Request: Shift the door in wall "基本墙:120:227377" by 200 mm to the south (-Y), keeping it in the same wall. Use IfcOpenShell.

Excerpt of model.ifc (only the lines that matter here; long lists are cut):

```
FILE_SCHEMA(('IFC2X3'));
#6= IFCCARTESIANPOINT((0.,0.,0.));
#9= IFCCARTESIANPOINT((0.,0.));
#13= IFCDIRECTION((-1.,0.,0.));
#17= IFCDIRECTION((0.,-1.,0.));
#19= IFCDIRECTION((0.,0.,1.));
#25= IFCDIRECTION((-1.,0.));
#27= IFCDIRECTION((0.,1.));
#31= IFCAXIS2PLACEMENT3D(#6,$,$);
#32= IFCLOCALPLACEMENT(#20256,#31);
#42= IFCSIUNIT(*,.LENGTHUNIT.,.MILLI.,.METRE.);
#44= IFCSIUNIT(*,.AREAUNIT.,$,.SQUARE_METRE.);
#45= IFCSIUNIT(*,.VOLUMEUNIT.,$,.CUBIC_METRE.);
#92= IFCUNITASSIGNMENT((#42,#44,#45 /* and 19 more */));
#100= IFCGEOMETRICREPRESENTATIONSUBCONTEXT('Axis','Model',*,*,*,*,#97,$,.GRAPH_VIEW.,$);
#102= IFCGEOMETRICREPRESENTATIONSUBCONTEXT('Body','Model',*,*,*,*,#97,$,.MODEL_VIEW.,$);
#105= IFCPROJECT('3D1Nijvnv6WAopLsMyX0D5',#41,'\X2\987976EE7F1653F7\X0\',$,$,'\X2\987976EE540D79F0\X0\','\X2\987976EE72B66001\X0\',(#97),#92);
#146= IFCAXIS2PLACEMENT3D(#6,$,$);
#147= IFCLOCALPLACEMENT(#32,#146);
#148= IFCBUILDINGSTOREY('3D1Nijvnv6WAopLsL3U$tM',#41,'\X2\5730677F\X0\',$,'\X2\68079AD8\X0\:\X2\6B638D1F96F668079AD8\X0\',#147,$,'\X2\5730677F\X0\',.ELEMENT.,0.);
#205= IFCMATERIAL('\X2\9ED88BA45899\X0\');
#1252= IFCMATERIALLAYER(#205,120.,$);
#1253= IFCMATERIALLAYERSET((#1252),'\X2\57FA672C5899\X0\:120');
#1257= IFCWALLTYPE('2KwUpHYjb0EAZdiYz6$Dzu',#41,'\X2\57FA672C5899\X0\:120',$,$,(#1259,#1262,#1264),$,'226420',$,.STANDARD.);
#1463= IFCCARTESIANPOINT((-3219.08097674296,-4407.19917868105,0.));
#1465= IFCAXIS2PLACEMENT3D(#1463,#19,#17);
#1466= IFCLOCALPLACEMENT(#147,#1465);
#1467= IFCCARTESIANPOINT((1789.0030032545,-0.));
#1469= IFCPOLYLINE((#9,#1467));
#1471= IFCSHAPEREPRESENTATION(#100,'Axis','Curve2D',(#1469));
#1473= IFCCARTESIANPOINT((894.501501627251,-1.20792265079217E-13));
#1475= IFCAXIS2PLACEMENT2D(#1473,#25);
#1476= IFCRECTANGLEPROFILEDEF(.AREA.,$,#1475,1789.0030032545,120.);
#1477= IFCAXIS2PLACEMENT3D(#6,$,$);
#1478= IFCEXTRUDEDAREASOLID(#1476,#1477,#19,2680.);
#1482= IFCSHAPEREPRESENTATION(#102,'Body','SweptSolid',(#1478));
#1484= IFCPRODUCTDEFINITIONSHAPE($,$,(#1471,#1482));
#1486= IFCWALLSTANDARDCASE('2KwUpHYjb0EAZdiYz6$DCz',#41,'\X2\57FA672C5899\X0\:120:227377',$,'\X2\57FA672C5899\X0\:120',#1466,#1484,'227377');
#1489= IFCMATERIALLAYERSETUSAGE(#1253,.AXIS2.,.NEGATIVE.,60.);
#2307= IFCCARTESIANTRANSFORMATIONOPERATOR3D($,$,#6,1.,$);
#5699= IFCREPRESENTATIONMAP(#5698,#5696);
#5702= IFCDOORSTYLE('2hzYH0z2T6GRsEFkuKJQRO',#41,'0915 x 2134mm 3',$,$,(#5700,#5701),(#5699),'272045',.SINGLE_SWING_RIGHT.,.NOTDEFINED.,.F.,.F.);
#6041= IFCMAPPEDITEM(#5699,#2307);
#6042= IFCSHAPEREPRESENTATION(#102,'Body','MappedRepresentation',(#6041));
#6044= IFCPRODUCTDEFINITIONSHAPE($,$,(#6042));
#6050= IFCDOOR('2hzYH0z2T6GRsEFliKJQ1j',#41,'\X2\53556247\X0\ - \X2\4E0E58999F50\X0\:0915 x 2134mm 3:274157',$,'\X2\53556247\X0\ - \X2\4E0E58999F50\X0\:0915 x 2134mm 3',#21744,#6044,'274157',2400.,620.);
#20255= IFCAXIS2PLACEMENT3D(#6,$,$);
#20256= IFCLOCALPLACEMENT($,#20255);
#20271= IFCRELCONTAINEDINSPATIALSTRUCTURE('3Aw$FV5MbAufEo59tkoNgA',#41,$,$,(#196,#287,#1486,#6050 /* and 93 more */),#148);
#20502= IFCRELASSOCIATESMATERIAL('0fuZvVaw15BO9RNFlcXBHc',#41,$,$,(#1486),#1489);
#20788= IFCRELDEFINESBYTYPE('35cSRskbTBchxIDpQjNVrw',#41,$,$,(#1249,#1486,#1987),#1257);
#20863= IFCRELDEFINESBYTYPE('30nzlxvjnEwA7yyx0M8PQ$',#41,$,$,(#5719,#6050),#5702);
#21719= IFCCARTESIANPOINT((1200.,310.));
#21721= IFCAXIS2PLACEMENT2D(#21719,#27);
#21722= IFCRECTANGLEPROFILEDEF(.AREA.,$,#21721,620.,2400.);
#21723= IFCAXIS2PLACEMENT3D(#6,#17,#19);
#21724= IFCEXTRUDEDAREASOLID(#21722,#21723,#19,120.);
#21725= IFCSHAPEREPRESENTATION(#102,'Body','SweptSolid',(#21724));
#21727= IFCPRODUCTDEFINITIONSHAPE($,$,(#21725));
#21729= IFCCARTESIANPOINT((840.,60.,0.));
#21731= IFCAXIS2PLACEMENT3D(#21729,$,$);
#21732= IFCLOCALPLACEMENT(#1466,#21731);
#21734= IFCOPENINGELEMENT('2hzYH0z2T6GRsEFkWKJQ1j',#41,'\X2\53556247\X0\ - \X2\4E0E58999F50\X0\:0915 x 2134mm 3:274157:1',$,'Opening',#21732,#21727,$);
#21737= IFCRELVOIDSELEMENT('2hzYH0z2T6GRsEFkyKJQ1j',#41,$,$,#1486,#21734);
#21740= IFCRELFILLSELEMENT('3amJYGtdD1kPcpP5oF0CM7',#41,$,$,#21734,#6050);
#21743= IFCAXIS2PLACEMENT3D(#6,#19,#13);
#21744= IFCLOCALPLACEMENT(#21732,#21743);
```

```python
import ifcopenshell
import ifcopenshell.api.geometry
import ifcopenshell.util.placement
import ifcopenshell.util.unit

model = ifcopenshell.open("model.ifc")
unit_scale = ifcopenshell.util.unit.calculate_unit_scale(model)

door = model.by_id(6050)
opening = door.FillsVoids[0].RelatingOpeningElement
wall = opening.VoidsElements[0].RelatingBuildingElement

wall_matrix = ifcopenshell.util.placement.get_local_placement(wall.ObjectPlacement)
shift = wall_matrix[:3, 0] * 0.2 / unit_scale
before = ifcopenshell.util.placement.get_local_placement(door.ObjectPlacement)[:3, 3].copy()

# The door is placed relative to its opening, so it follows when the opening moves.
matrix = ifcopenshell.util.placement.get_local_placement(opening.ObjectPlacement)
matrix[:3, 3] += shift
ifcopenshell.api.geometry.edit_object_placement(
    model, product=opening, matrix=matrix, is_si=False, should_transform_children=True
)

after = ifcopenshell.util.placement.get_local_placement(door.ObjectPlacement)[:3, 3]
print("door moved by", (after - before).round(3) + 0.0)

model.write("model_rev.ifc")
```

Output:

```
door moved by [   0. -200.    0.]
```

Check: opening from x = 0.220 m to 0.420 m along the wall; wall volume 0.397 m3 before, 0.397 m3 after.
